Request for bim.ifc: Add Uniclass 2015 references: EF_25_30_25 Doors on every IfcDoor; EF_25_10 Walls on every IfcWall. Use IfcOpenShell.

First a look at what the model holds.

```python
import ifcopenshell

model = ifcopenshell.open("bim.ifc")
print(model.schema)
print("classifications:", [c.Name for c in model.by_type("IfcClassification")])
for ifc_class in ("IfcDoor", "IfcRoof", "IfcStair", "IfcWall", "IfcWindow"):
    print(ifc_class, len(model.by_type(ifc_class)))
```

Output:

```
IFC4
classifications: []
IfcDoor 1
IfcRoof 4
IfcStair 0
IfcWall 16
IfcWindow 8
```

```python
import ifcopenshell
import ifcopenshell.api.classification

model = ifcopenshell.open("bim.ifc")

system = ifcopenshell.api.classification.add_classification(model, classification="Uniclass 2015")

codes = {
    "IfcDoor": ("EF_25_30_25", "Doors"),
    "IfcWall": ("EF_25_10", "Walls"),
}
for ifc_class, (code, name) in codes.items():
    products = model.by_type(ifc_class)
    ifcopenshell.api.classification.add_reference(
        model, products=products, classification=system, identification=code, name=name
    )
    print(code, len(products))

model.write("bim_rev.ifc")
```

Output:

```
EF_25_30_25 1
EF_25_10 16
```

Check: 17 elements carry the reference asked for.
